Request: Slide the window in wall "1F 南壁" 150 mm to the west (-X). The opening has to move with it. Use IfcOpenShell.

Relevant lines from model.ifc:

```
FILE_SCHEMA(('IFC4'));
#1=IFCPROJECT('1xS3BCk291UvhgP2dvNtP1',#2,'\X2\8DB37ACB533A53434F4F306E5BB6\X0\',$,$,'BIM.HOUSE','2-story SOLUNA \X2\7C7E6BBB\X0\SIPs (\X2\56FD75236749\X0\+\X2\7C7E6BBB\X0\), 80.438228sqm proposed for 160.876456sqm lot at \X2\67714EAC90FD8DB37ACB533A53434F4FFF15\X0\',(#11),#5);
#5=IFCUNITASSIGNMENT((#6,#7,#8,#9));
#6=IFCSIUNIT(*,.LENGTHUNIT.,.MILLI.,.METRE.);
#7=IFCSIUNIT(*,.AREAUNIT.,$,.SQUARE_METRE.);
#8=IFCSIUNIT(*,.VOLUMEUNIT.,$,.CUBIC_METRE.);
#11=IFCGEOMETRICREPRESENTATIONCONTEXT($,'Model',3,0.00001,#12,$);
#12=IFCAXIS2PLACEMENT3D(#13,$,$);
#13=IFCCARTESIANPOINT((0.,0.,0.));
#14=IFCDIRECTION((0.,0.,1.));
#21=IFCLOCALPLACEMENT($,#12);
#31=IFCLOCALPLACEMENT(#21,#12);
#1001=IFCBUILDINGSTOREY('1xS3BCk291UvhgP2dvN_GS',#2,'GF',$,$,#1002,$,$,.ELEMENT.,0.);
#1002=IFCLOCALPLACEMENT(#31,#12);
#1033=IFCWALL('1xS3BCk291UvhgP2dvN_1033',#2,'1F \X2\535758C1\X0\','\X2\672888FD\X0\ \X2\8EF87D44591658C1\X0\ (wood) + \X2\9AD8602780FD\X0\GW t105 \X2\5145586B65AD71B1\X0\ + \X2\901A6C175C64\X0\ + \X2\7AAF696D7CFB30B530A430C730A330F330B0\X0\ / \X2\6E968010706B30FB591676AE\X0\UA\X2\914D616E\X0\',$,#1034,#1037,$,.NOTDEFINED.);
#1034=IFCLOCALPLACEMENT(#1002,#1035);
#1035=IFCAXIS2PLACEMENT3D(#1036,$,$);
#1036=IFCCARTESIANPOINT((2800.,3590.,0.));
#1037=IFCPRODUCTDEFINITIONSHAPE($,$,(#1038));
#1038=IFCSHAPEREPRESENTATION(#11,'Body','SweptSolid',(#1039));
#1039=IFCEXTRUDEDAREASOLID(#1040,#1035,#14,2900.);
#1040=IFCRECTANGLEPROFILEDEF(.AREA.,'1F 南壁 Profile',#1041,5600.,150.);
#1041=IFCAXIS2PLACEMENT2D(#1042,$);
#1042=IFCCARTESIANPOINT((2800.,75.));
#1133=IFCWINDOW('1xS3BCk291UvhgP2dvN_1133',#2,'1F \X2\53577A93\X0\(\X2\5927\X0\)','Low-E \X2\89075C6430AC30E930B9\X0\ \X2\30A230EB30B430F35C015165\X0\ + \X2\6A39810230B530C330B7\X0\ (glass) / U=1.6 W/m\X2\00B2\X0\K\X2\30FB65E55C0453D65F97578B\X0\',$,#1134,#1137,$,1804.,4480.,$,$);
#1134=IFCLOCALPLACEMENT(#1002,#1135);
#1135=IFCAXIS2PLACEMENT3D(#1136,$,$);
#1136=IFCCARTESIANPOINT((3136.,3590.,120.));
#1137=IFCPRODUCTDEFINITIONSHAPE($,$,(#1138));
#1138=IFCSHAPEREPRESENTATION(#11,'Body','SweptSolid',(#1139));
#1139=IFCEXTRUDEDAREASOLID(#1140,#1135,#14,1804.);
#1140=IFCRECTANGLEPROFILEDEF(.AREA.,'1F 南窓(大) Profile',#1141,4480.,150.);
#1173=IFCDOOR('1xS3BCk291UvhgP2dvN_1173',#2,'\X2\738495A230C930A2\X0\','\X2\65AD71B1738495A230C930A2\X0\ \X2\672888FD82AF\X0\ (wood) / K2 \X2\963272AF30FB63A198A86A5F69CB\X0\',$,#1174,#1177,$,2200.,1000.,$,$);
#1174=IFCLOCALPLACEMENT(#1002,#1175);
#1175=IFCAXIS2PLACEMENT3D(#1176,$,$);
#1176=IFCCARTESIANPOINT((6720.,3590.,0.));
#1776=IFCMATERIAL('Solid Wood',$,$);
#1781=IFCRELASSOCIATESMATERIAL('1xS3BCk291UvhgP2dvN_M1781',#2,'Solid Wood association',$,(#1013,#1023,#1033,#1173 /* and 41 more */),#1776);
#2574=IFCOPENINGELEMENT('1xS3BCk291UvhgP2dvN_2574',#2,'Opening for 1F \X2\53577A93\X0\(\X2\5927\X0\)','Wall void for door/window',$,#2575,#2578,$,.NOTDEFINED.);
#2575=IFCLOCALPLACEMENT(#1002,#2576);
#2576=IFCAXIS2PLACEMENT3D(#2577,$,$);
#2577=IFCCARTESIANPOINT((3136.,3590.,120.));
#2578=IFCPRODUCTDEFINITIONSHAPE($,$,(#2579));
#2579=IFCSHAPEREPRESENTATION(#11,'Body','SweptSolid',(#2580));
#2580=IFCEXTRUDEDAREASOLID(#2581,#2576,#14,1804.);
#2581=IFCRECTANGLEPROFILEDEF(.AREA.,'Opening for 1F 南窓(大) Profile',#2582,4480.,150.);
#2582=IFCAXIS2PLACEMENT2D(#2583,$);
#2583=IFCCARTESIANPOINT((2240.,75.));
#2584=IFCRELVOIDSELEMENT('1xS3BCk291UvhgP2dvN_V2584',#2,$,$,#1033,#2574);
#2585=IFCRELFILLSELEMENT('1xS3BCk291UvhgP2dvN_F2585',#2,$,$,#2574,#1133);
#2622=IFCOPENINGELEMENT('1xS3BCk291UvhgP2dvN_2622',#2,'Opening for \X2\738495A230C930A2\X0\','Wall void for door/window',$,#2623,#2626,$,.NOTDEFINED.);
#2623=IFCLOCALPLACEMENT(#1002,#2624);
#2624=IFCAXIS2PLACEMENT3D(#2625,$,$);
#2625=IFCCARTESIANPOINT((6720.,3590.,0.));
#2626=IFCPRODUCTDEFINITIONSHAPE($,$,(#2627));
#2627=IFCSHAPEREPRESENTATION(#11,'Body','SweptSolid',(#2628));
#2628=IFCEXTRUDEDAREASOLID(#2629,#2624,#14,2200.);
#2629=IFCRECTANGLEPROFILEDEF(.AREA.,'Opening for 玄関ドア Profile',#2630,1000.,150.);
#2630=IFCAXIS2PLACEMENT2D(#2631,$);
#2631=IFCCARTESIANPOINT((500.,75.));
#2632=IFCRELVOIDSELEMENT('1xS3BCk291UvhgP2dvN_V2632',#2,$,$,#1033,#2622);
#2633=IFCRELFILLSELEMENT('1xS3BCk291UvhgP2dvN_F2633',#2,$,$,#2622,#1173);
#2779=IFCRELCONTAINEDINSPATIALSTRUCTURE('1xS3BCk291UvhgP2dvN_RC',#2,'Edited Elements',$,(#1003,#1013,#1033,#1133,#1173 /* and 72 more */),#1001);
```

```python
import ifcopenshell
import ifcopenshell.api.geometry
import ifcopenshell.util.placement

model = ifcopenshell.open("model.ifc")

window = model.by_guid("1xS3BCk291UvhgP2dvN_1133")
opening = window.FillsVoids[0].RelatingOpeningElement
wall = opening.VoidsElements[0].RelatingBuildingElement

wall_matrix = ifcopenshell.util.placement.get_local_placement(wall.ObjectPlacement)
shift = wall_matrix[:3, 0] * -150.0
before = ifcopenshell.util.placement.get_local_placement(window.ObjectPlacement)[:3, 3].copy()

# The window is not placed relative to its opening, so move both.
for product in (opening, window):
    matrix = ifcopenshell.util.placement.get_local_placement(product.ObjectPlacement)
    matrix[:3, 3] += shift
    ifcopenshell.api.geometry.edit_object_placement(model, product=product, matrix=matrix, is_si=False)

after = ifcopenshell.util.placement.get_local_placement(window.ObjectPlacement)[:3, 3]
print("window moved by", (after - before).round(3) + 0.0)

model.write("model_edited.ifc")
```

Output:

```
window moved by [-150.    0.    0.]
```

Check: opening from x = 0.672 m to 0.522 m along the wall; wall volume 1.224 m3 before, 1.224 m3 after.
